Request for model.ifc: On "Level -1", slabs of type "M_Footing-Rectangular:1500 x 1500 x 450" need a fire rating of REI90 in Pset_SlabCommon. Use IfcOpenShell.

First a look at what the model holds.

```python
import ifcopenshell
import ifcopenshell.util.element

model = ifcopenshell.open("model.ifc")
print(model.schema)
storey = next(s for s in model.by_type("IfcBuildingStorey") if s.Name == "Level -1")
slabs = [e for e in ifcopenshell.util.element.get_decomposition(storey) if e.is_a("IfcSlab")]
seen = {}
for e in slabs:
    element_type = ifcopenshell.util.element.get_type(e)
    key = (element_type.Name if element_type != e and element_type else None, ifcopenshell.util.element.get_pset(e, "Pset_SlabCommon", "FireRating"))
    seen[key] = seen.get(key, 0) + 1
for (name, value), count in sorted(seen.items(), key=str):
    print(count, "x", name, "|", value)
```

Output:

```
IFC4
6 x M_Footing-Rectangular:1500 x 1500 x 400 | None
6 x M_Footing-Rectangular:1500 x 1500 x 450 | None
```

```python
import ifcopenshell
import ifcopenshell.api.pset
import ifcopenshell.util.element

model = ifcopenshell.open("model.ifc")

storey = next(s for s in model.by_type("IfcBuildingStorey") if s.Name == "Level -1")
slabs = [e for e in ifcopenshell.util.element.get_decomposition(storey) if e.is_a("IfcSlab")]

count = 0
for e in slabs:
    element_type = ifcopenshell.util.element.get_type(e)
    if element_type in (None, e) or element_type.Name != "M_Footing-Rectangular:1500 x 1500 x 450":
        continue
    # add_pset returns the element's existing set when there is one.
    pset = ifcopenshell.api.pset.add_pset(model, product=e, name="Pset_SlabCommon")
    ifcopenshell.api.pset.edit_pset(model, pset=pset, properties={"FireRating": "REI90"})
    count += 1

print(count, "slabs updated")

model.write("model_v2.ifc")
```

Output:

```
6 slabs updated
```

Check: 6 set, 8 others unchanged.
